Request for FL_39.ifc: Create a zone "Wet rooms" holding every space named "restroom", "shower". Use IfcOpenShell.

First a look at what the model holds.

```python
import ifcopenshell

model = ifcopenshell.open("FL_39.ifc")
print(model.schema)
seen = {}
for space in model.by_type("IfcSpace"):
    seen[space.LongName] = seen.get(space.LongName, 0) + 1
for name, count in sorted(seen.items(), key=str):
    print(count, "x", name)
print("zones:", [z.Name for z in model.by_type("IfcZone")][:20])
```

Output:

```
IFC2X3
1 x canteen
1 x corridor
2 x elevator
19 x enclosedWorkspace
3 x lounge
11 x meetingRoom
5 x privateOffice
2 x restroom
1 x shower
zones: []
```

```python
import ifcopenshell
import ifcopenshell.api.group
import ifcopenshell.api.root

model = ifcopenshell.open("FL_39.ifc")

names = {"restroom", "shower"}
spaces = [s for s in model.by_type("IfcSpace") if s.LongName in names]

zone = ifcopenshell.api.root.create_entity(model, ifc_class="IfcZone", name="Wet rooms")
ifcopenshell.api.group.assign_group(model, products=spaces, group=zone)
print(len(spaces), "spaces in", zone.Name)

model.write("FL_39_v2.ifc")
```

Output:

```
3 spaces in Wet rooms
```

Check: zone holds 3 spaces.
